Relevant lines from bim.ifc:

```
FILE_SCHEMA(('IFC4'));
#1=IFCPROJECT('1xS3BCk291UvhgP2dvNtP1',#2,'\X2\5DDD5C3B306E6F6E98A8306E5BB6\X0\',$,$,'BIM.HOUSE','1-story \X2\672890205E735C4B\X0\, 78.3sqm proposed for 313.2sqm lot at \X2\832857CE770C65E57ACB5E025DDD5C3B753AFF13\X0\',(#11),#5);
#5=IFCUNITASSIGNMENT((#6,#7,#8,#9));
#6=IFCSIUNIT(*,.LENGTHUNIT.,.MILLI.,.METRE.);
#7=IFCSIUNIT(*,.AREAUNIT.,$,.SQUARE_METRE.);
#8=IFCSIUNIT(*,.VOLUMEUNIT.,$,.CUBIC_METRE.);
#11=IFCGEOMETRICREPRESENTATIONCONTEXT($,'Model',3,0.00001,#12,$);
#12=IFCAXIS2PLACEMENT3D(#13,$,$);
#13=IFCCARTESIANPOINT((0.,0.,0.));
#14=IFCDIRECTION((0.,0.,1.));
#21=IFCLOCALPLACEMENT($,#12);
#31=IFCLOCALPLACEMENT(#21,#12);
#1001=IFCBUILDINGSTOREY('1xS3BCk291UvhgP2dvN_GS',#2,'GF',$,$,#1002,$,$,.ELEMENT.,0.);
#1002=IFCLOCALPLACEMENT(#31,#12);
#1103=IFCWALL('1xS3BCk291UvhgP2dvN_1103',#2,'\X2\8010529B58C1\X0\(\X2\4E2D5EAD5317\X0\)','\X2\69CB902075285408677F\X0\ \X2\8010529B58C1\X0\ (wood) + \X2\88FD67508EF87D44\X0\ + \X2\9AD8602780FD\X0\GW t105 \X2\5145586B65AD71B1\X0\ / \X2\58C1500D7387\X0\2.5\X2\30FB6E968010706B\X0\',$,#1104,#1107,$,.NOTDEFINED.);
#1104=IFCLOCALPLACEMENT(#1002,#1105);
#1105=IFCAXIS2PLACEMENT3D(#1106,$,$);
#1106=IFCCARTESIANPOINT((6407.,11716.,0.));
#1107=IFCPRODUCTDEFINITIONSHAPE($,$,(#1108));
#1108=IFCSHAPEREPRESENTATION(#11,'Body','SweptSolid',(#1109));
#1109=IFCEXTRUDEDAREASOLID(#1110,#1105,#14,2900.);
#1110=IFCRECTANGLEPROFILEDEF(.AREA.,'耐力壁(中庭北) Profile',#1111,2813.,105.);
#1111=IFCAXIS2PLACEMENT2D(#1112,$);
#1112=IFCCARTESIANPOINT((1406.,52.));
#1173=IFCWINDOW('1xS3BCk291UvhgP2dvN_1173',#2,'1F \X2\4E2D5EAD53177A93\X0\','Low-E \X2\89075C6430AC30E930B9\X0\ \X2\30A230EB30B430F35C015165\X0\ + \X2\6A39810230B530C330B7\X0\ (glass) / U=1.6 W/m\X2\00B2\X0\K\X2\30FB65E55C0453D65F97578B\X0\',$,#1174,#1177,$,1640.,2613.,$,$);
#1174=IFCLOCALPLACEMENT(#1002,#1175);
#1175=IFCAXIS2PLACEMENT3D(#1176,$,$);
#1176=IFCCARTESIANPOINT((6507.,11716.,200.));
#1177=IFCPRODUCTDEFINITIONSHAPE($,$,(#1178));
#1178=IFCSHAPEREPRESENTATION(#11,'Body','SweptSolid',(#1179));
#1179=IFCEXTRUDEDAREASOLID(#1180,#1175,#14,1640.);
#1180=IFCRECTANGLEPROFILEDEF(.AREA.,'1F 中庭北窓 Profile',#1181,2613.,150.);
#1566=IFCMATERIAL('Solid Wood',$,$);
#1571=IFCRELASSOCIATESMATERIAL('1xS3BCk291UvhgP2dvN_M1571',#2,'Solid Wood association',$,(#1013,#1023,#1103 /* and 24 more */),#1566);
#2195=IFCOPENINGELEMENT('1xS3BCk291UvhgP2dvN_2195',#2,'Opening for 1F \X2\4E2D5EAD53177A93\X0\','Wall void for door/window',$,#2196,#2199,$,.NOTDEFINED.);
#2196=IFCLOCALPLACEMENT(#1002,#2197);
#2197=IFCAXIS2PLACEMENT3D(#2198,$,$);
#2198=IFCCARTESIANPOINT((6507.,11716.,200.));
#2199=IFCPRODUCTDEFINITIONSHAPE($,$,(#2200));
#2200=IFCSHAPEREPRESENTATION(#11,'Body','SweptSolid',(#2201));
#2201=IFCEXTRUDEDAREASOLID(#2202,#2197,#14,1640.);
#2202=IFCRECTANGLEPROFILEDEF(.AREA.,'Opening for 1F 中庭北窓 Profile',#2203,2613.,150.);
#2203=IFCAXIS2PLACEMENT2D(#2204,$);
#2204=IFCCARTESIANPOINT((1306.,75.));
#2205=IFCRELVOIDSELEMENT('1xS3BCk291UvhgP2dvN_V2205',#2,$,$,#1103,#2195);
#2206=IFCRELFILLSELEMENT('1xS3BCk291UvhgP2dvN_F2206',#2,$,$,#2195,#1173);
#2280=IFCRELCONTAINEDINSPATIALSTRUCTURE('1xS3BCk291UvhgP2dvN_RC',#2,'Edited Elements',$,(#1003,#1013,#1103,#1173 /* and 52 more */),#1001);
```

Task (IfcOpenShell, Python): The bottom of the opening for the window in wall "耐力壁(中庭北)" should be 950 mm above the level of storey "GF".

```python
import numpy as np
import ifcopenshell
import ifcopenshell.api.geometry
import ifcopenshell.geom
import ifcopenshell.util.element
import ifcopenshell.util.placement
import ifcopenshell.util.shape
import ifcopenshell.util.unit

model = ifcopenshell.open("bim.ifc")
unit_scale = ifcopenshell.util.unit.calculate_unit_scale(model)

window = model.by_guid("1xS3BCk291UvhgP2dvN_1173")
opening = window.FillsVoids[0].RelatingOpeningElement
storey = ifcopenshell.util.element.get_container(window, ifc_class="IfcBuildingStorey")
level = ifcopenshell.util.placement.get_local_placement(storey.ObjectPlacement)[2, 3]

# The opening's origin need not be at the sill, so measure its lowest point.
shape = ifcopenshell.geom.create_shape(ifcopenshell.geom.settings(), opening)
bottom = ifcopenshell.util.shape.get_shape_bottom_elevation(shape, shape.geometry) / unit_scale
dz = level + 0.95 / unit_scale - bottom

shift = np.array([0.0, 0.0, dz])
# The window is not placed relative to its opening, so move both.
for product in (opening, window):
    matrix = ifcopenshell.util.placement.get_local_placement(product.ObjectPlacement)
    matrix[:3, 3] += shift
    ifcopenshell.api.geometry.edit_object_placement(model, product=product, matrix=matrix, is_si=False)

print(f"moved by {dz * unit_scale:+.3f} m")

model.write("bim_rev.ifc")
```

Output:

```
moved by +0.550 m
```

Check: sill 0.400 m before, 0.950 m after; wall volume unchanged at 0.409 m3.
